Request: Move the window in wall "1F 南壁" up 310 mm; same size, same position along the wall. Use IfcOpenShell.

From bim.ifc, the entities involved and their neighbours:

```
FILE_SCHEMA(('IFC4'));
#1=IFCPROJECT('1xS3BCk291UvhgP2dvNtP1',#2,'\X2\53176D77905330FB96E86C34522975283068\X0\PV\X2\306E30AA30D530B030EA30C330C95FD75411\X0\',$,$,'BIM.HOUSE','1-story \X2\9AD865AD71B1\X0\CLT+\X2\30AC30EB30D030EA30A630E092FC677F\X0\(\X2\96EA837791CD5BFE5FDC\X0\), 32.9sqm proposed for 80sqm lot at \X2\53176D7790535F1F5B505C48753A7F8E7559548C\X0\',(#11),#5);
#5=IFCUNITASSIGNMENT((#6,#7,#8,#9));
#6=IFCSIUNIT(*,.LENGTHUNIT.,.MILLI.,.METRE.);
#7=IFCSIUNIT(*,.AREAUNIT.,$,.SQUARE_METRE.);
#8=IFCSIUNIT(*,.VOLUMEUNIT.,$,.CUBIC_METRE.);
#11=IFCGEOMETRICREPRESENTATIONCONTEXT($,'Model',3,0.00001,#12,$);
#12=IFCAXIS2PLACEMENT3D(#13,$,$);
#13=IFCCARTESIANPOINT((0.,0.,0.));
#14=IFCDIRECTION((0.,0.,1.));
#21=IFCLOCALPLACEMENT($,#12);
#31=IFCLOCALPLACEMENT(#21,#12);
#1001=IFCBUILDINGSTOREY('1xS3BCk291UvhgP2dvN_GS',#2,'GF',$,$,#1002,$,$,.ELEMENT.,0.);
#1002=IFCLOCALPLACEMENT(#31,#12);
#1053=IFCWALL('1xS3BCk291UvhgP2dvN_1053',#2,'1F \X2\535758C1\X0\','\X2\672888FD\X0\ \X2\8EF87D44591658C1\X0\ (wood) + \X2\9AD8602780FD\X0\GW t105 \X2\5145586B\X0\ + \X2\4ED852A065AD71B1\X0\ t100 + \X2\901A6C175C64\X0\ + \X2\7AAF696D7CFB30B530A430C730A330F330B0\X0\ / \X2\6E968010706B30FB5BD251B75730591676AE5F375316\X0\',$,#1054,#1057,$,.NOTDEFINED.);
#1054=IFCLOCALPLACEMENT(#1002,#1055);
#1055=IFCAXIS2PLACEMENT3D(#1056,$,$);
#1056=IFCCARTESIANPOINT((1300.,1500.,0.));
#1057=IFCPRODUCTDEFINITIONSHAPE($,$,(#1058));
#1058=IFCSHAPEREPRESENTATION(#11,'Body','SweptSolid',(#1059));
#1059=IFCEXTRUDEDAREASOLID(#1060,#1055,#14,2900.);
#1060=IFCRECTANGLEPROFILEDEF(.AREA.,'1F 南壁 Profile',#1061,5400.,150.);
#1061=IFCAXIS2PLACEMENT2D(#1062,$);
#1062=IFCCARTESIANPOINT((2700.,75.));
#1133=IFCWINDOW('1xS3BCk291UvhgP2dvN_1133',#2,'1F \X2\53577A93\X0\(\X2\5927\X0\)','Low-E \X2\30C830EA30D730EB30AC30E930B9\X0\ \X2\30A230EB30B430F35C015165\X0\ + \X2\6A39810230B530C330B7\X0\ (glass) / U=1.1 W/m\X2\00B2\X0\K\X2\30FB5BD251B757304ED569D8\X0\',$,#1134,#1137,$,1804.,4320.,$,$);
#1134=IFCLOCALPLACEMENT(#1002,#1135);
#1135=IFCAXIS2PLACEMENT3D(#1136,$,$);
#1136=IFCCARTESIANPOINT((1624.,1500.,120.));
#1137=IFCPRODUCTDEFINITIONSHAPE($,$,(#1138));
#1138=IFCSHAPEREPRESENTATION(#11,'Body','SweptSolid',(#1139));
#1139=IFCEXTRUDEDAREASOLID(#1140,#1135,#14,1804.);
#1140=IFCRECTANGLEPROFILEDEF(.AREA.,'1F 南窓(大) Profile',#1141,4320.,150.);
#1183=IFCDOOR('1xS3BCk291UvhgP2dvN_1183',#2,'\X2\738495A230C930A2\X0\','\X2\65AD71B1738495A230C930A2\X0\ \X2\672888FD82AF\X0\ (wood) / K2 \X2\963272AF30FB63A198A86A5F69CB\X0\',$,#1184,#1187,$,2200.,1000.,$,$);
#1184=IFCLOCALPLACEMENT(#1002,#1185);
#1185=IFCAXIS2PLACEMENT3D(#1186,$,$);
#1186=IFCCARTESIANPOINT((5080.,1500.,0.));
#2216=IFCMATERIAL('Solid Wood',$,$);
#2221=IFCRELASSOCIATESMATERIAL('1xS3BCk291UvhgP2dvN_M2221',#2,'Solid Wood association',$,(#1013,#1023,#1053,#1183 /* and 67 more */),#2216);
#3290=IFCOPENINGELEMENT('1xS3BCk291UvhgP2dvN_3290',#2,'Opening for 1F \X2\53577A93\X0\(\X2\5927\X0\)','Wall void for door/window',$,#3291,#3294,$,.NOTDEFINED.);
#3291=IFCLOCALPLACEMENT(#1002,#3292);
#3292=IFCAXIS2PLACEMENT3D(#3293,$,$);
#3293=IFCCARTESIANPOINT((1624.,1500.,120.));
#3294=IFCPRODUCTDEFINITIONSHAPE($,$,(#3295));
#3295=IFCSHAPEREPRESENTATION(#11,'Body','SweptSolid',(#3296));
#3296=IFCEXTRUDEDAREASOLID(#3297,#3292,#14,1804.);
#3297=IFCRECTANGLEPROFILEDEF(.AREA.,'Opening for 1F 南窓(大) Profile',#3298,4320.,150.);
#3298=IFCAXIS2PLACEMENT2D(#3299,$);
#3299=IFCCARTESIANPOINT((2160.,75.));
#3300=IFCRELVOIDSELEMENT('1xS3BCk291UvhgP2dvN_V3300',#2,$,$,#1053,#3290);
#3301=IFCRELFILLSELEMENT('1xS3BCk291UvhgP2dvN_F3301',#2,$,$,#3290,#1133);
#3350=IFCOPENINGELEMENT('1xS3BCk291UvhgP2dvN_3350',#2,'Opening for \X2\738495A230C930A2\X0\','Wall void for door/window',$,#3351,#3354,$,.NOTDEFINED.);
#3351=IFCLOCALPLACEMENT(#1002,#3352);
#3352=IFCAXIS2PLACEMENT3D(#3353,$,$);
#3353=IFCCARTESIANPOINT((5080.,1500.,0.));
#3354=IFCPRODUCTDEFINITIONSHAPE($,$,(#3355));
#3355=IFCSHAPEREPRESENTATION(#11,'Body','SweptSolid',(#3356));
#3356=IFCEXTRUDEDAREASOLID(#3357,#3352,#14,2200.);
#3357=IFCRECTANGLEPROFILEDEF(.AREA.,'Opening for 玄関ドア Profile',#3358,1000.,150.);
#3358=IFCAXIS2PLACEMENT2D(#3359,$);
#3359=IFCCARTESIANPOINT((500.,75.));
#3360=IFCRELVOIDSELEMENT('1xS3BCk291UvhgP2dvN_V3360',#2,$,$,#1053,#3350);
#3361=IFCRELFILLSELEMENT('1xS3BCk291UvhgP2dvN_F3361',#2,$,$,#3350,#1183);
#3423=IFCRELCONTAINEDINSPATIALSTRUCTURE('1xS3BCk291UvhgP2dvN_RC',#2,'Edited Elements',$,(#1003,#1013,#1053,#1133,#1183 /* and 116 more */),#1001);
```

```python
import numpy as np
import ifcopenshell
import ifcopenshell.api.geometry
import ifcopenshell.util.placement
import ifcopenshell.util.unit

model = ifcopenshell.open("bim.ifc")
unit_scale = ifcopenshell.util.unit.calculate_unit_scale(model)

window = model.by_guid("1xS3BCk291UvhgP2dvN_1133")
opening = window.FillsVoids[0].RelatingOpeningElement
dz = 310.0

shift = np.array([0.0, 0.0, dz])
# The window is not placed relative to its opening, so move both.
for product in (opening, window):
    matrix = ifcopenshell.util.placement.get_local_placement(product.ObjectPlacement)
    matrix[:3, 3] += shift
    ifcopenshell.api.geometry.edit_object_placement(model, product=product, matrix=matrix, is_si=False)

print(f"moved by {dz * unit_scale:+.3f} m")

model.write("bim_updated.ifc")
```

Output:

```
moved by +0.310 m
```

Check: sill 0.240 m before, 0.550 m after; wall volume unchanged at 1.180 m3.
